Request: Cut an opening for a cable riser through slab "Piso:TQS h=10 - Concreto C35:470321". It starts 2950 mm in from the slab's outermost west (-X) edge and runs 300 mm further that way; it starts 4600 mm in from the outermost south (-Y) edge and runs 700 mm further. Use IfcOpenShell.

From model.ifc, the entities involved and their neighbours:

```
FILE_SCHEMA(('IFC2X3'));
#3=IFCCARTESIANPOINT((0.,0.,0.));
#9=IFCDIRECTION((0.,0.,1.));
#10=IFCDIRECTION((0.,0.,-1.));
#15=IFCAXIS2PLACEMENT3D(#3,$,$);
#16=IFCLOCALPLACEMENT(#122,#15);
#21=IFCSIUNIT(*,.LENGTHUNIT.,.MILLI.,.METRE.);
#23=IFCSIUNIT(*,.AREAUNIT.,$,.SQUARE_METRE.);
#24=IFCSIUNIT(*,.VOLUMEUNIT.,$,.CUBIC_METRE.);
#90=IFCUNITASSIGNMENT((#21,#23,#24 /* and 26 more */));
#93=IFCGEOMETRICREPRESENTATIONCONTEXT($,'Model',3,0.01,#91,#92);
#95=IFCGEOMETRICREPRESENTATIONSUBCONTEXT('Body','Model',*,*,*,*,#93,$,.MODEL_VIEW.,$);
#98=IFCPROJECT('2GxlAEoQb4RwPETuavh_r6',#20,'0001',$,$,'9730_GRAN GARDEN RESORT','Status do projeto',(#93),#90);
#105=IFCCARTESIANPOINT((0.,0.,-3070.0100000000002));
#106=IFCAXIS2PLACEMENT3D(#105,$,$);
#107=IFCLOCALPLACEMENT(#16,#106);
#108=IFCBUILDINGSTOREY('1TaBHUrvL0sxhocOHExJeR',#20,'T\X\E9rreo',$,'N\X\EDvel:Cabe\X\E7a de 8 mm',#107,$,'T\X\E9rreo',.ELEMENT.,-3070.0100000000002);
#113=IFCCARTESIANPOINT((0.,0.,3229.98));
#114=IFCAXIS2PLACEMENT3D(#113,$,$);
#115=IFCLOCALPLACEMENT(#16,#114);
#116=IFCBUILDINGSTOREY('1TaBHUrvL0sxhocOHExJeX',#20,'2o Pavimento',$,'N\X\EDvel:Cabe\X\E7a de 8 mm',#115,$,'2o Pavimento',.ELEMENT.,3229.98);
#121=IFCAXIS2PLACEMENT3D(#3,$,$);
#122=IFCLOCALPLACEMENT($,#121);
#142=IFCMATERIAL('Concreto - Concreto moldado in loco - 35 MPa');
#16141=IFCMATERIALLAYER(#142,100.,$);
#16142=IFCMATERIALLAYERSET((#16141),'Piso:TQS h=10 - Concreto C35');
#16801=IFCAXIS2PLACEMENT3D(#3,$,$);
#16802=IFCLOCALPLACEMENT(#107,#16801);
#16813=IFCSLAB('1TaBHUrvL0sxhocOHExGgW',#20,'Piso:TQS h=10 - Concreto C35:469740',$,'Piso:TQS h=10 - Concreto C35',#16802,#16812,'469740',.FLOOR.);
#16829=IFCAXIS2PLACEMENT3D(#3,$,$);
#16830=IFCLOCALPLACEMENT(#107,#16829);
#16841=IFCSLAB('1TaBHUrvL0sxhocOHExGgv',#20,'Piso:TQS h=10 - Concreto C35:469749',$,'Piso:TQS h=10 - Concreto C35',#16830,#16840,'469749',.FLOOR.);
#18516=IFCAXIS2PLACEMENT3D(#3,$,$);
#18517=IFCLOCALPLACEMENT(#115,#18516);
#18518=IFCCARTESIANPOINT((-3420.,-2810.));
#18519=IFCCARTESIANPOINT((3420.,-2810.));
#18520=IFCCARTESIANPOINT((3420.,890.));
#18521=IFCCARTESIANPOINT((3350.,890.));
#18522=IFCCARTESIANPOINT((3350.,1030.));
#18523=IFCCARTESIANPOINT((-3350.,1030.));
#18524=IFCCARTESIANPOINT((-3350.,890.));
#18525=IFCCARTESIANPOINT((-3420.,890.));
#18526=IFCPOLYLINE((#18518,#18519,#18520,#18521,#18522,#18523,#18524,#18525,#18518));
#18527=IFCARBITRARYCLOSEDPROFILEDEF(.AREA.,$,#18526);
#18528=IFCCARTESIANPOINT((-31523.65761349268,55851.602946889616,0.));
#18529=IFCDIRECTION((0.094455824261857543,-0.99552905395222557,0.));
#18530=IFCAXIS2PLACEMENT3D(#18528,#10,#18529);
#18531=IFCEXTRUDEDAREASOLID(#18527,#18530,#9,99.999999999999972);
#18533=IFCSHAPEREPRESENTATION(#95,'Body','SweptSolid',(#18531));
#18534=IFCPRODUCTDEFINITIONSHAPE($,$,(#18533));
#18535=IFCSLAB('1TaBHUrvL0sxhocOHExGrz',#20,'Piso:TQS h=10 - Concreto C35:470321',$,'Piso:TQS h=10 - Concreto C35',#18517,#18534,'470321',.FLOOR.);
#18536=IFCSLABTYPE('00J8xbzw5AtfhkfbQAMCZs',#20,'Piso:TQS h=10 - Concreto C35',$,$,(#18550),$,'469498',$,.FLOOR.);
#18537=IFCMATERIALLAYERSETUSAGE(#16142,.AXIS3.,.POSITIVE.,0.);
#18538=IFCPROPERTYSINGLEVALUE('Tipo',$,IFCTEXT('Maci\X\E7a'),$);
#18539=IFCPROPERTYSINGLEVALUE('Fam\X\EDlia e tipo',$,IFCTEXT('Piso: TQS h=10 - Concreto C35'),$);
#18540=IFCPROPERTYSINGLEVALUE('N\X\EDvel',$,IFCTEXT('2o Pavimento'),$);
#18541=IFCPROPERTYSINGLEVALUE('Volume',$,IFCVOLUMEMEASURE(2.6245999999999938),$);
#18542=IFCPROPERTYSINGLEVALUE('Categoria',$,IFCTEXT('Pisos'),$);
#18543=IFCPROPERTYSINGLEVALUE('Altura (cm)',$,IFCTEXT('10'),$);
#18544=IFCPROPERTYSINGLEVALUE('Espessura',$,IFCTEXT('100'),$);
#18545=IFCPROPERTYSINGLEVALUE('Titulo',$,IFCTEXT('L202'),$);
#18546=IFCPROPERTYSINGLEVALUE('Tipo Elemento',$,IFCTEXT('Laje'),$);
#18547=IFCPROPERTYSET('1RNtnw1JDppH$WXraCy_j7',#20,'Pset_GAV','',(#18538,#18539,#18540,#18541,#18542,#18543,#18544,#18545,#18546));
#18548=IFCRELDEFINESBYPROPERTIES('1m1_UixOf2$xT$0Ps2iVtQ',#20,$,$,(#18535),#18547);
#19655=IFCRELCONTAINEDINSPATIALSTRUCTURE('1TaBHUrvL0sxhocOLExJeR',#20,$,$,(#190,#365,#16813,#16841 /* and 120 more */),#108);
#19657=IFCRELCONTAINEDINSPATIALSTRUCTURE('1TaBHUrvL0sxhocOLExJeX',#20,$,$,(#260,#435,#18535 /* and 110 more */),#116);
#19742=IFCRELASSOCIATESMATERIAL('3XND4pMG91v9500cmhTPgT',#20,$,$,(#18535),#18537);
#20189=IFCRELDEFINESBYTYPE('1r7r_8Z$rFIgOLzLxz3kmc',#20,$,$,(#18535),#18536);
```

```python
import numpy as np
import ifcopenshell
import ifcopenshell.api.feature
import ifcopenshell.api.geometry
import ifcopenshell.api.pset
import ifcopenshell.api.root
import ifcopenshell.geom
import ifcopenshell.util.element
import ifcopenshell.util.placement
import ifcopenshell.util.representation
import ifcopenshell.util.shape
import ifcopenshell.util.unit

model = ifcopenshell.open("model.ifc")
unit_scale = ifcopenshell.util.unit.calculate_unit_scale(model)
volume_scale = ifcopenshell.util.unit.calculate_unit_scale(model, "VOLUMEUNIT")
settings = ifcopenshell.geom.settings()


def volume(element):
    """Net volume in cubic metres, openings subtracted."""
    shape = ifcopenshell.geom.create_shape(settings, element)
    return ifcopenshell.util.shape.get_volume(shape.geometry)


slab = model.by_guid("1TaBHUrvL0sxhocOHExGrz")
before = volume(slab)

# Extent in the slab's own axes, in metres. The edges named are its -X and -Y sides.
slab_shape = ifcopenshell.geom.create_shape(settings, slab)
vertices = ifcopenshell.util.shape.get_vertices(slab_shape.geometry)
x_min, y_min, bottom = vertices.min(axis=0)
top = vertices[:, 2].max()

opening = ifcopenshell.api.root.create_entity(model, ifc_class="IfcOpeningElement", name="Cable riser opening")
context = ifcopenshell.util.representation.get_context(model, "Model", "Body", "MODEL_VIEW")
width, depth = 0.3, 0.7
outline = [(0.0, 0.0), (width, 0.0), (width, depth), (0.0, depth), (0.0, 0.0)]
# Overshoot both faces by 50 mm so the cut is clean.
shape = ifcopenshell.api.geometry.add_slab_representation(
    model, context=context, depth=top - bottom + 0.1, polyline=outline
)
ifcopenshell.api.geometry.assign_representation(model, product=opening, representation=shape)

matrix = ifcopenshell.util.placement.get_local_placement(slab.ObjectPlacement)
matrix[:, 3] = matrix @ np.append(np.array([x_min + 2.95, y_min + 4.6, bottom - 0.05]) / unit_scale, 1.0)
ifcopenshell.api.geometry.edit_object_placement(model, product=opening, matrix=matrix, is_si=False)
ifcopenshell.api.feature.add_feature(model, feature=opening, element=slab)

after = volume(slab)

# Update the slab's stored quantities.
pset = model.by_id(ifcopenshell.util.element.get_pset(slab, "Pset_GAV", should_inherit=False)["id"])
ifcopenshell.api.pset.edit_pset(model, pset=pset, properties={
    "Volume": model.create_entity("IfcVolumeMeasure", after / volume_scale),
})

print(f"slab volume {before:.3f} -> {after:.3f} m3")

model.write("model_updated.ifc")
```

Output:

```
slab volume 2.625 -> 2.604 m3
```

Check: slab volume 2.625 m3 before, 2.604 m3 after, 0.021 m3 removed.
